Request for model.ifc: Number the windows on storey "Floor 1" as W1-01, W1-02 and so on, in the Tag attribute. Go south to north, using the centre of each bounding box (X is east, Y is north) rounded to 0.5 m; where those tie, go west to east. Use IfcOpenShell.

First a look at what the model holds.

```python
import ifcopenshell
import ifcopenshell.util.element
import ifcopenshell.util.placement

model = ifcopenshell.open("model.ifc")
print(model.schema)
storey = next(s for s in model.by_type("IfcBuildingStorey") if s.Name == "Floor 1")
windows = [e for e in ifcopenshell.util.element.get_decomposition(storey) if e.is_a("IfcWindow")]
for e in sorted(windows, key=lambda e: e.id()):
    origin = ifcopenshell.util.placement.get_local_placement(e.ObjectPlacement)[:3, 3]
    print(e.id(), e.Tag, e.Name, origin.round(2) + 0.0, sep=" | ")
```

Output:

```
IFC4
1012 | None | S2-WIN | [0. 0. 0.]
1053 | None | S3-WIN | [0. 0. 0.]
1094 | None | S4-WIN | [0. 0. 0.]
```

```python
import ifcopenshell
import ifcopenshell.geom
import ifcopenshell.util.element
import ifcopenshell.util.shape

model = ifcopenshell.open("model.ifc")
settings = ifcopenshell.geom.settings()
settings.set("use-world-coords", True)


def centre(element):
    shape = ifcopenshell.geom.create_shape(settings, element)
    return ifcopenshell.util.shape.get_bbox_centroid(shape.geometry)


storey = next(s for s in model.by_type("IfcBuildingStorey") if s.Name == "Floor 1")
windows = [e for e in ifcopenshell.util.element.get_decomposition(storey) if e.is_a("IfcWindow")]

# Insertion points can sit at a corner or the storey origin, so sort by the geometry (in metres).
centres = {e: centre(e) for e in windows}
windows.sort(key=lambda e: (round(centres[e][1] / 0.5), centres[e][0]))

for i, e in enumerate(windows, start=1):
    number = f"W1-{i:02d}"
    e.Tag = number
    print(e.id(), number)

model.write("model-out.ifc")
```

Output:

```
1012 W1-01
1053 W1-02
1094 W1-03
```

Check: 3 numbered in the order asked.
